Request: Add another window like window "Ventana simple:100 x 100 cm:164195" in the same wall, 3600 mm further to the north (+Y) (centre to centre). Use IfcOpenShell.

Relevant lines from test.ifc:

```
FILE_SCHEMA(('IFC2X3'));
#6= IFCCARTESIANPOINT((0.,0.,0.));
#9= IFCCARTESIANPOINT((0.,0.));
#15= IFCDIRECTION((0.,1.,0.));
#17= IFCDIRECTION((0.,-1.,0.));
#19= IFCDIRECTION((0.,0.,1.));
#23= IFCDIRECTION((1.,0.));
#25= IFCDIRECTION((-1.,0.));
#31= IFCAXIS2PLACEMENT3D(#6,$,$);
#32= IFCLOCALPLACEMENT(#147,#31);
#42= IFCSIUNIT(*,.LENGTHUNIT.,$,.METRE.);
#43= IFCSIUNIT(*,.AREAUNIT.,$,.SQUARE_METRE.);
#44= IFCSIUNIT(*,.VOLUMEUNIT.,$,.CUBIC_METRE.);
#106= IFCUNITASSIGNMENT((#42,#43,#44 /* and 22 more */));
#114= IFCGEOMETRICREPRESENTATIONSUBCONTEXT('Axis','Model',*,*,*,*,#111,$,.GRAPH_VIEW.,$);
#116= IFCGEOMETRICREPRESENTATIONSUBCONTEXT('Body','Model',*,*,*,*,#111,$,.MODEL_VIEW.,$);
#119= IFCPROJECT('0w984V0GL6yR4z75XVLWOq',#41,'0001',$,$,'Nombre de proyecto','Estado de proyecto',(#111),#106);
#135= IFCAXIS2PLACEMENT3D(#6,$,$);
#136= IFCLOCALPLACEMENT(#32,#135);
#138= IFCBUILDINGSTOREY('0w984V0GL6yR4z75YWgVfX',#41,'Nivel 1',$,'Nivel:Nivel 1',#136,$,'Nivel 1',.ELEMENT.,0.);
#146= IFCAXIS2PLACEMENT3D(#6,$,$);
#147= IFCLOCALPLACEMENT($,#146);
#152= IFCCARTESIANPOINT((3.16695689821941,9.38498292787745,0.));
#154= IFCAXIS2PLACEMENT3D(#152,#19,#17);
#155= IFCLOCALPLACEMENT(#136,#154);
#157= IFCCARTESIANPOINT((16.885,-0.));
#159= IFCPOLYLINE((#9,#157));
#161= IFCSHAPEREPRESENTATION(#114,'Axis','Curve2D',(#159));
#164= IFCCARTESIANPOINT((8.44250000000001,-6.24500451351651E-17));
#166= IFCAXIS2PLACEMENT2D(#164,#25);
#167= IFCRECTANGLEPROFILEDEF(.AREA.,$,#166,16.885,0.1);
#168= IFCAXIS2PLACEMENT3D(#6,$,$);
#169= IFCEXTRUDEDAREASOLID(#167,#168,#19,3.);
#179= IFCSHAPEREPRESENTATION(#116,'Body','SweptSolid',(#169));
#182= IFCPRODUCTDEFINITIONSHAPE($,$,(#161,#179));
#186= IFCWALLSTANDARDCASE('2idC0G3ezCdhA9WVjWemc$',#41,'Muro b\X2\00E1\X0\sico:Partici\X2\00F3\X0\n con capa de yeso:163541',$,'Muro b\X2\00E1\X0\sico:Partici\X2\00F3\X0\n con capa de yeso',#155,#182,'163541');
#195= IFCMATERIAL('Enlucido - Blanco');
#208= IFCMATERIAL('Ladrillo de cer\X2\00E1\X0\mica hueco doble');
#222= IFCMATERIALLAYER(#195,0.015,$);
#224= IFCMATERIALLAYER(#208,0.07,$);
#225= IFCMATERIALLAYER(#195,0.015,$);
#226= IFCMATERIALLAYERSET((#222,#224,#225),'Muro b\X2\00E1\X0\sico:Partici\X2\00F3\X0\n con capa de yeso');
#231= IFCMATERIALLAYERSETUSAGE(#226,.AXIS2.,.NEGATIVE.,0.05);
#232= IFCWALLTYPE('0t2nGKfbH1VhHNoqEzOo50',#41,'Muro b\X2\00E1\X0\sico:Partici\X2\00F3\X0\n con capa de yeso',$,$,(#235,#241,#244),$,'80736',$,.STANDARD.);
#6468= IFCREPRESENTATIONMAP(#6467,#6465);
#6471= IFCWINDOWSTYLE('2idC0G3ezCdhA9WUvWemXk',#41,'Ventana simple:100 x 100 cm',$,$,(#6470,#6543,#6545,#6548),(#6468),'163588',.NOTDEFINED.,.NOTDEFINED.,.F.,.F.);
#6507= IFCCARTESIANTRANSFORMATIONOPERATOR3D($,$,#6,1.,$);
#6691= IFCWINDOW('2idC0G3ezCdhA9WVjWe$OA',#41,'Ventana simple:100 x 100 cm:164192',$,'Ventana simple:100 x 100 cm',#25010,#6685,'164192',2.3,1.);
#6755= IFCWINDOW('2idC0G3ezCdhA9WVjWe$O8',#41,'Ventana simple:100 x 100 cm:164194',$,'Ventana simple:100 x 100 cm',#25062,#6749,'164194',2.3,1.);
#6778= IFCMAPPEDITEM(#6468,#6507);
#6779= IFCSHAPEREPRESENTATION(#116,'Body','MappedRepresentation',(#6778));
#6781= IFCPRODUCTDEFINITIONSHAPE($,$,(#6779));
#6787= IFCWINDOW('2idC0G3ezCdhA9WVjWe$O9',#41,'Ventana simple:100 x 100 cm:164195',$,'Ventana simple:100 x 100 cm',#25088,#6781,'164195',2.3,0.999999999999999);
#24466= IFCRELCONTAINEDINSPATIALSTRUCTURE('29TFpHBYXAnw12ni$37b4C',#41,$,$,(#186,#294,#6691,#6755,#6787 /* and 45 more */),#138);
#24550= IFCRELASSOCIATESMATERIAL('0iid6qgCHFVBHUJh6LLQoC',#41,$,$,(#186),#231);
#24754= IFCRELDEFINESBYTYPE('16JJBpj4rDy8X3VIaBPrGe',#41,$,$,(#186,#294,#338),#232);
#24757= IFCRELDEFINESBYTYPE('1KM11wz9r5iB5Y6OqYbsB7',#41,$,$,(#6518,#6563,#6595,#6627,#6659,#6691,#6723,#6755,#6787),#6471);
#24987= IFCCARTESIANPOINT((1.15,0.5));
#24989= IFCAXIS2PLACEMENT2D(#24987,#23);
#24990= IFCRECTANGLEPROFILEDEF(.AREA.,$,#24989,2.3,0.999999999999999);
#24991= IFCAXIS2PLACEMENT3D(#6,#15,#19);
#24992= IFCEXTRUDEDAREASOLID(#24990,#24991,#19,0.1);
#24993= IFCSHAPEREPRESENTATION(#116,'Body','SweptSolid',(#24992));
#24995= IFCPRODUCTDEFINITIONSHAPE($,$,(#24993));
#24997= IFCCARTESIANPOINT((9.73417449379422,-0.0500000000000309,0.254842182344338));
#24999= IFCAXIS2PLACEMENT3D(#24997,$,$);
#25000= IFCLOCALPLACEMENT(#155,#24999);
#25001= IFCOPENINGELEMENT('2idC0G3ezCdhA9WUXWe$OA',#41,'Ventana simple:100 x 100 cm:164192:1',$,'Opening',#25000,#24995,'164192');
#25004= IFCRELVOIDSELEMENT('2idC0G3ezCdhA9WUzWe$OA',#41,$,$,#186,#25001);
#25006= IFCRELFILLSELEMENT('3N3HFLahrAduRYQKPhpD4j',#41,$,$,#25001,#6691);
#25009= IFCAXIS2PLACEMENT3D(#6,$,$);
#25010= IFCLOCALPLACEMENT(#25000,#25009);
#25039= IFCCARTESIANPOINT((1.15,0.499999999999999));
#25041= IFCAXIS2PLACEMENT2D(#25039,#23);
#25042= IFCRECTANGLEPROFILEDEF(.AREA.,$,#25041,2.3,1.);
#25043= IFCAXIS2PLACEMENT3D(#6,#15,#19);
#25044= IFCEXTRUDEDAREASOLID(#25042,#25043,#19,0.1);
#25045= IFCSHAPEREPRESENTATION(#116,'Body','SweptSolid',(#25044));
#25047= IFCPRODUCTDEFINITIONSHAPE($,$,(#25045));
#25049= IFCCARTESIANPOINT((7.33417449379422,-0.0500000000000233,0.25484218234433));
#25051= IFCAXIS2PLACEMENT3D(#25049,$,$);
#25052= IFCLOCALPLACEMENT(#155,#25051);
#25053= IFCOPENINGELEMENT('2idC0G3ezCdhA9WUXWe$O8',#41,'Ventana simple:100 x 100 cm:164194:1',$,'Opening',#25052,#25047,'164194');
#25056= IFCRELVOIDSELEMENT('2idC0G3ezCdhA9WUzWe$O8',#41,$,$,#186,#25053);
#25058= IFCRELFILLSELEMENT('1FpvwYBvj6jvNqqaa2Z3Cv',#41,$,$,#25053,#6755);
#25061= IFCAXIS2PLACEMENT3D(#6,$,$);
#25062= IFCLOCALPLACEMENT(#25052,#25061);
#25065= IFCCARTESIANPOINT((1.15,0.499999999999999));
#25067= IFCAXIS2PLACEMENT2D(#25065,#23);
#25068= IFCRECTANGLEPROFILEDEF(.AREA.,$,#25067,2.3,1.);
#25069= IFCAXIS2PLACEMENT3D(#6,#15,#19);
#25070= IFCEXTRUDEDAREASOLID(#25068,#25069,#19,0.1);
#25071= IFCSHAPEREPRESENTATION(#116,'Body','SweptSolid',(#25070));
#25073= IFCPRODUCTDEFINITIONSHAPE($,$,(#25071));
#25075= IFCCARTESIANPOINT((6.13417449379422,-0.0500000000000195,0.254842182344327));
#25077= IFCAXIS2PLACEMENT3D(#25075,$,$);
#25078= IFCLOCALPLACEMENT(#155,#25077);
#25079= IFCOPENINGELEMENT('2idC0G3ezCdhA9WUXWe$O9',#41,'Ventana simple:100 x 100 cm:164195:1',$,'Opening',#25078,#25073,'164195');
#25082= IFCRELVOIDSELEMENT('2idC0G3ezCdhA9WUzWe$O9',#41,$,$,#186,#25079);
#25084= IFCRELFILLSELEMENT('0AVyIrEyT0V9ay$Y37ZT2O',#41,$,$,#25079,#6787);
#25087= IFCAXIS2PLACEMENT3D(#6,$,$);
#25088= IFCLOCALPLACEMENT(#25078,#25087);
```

```python
import ifcopenshell
import ifcopenshell.api.feature
import ifcopenshell.api.geometry
import ifcopenshell.api.root
import ifcopenshell.geom
import ifcopenshell.util.element
import ifcopenshell.util.placement
import ifcopenshell.util.shape

model = ifcopenshell.open("test.ifc")
settings = ifcopenshell.geom.settings()


def volume(element):
    """Net volume in cubic metres, openings subtracted."""
    shape = ifcopenshell.geom.create_shape(settings, element)
    return ifcopenshell.util.shape.get_volume(shape.geometry)


def reuse_history(source, copy):
    """copy_class also copies each property set's owner history, people and application; keep the originals."""
    for rel in copy.IsDefinedBy:
        if rel.is_a("IfcRelDefinesByProperties") and (history := rel.RelatingPropertyDefinition.OwnerHistory):
            rel.RelatingPropertyDefinition.OwnerHistory = source.OwnerHistory
            ifcopenshell.util.element.remove_deep2(model, history)


window = model.by_guid("2idC0G3ezCdhA9WVjWe$O9")
opening = window.FillsVoids[0].RelatingOpeningElement
wall = opening.VoidsElements[0].RelatingBuildingElement
before = volume(wall)
shift = ifcopenshell.util.placement.get_local_placement(wall.ObjectPlacement)[:3, 0] * -3.6

# copy_class copies the void relationship, type, container and properties, but no geometry.
new_opening = ifcopenshell.api.root.copy_class(model, product=opening)
new_opening.Representation = ifcopenshell.util.element.copy_deep(
    model, opening.Representation, exclude=["IfcGeometricRepresentationContext", "IfcRepresentationMap"]
)
new_opening.Name = "Ventana simple:100 x 100 cm"
new_opening.Tag = None
new_window = ifcopenshell.api.root.copy_class(model, product=window)
new_window.Representation = ifcopenshell.util.element.copy_deep(
    model, window.Representation, exclude=["IfcGeometricRepresentationContext", "IfcRepresentationMap"]
)
new_window.Name = "Ventana simple:100 x 100 cm"
new_window.Tag = None
reuse_history(window, new_window)
fills = ifcopenshell.api.feature.add_filling(model, opening=new_opening, element=new_window)
fills.OwnerHistory = new_window.OwnerHistory  # required in IFC2X3

for old, new in ((opening, new_opening), (window, new_window)):
    matrix = ifcopenshell.util.placement.get_local_placement(old.ObjectPlacement)
    matrix[:3, 3] += shift
    ifcopenshell.api.geometry.edit_object_placement(model, product=new, matrix=matrix, is_si=False)

after = volume(wall)

print(f"wall volume {before:.3f} -> {after:.3f} m3")

model.write("test_updated.ifc")
```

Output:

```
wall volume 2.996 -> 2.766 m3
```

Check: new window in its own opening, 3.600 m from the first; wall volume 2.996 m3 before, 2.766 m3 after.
